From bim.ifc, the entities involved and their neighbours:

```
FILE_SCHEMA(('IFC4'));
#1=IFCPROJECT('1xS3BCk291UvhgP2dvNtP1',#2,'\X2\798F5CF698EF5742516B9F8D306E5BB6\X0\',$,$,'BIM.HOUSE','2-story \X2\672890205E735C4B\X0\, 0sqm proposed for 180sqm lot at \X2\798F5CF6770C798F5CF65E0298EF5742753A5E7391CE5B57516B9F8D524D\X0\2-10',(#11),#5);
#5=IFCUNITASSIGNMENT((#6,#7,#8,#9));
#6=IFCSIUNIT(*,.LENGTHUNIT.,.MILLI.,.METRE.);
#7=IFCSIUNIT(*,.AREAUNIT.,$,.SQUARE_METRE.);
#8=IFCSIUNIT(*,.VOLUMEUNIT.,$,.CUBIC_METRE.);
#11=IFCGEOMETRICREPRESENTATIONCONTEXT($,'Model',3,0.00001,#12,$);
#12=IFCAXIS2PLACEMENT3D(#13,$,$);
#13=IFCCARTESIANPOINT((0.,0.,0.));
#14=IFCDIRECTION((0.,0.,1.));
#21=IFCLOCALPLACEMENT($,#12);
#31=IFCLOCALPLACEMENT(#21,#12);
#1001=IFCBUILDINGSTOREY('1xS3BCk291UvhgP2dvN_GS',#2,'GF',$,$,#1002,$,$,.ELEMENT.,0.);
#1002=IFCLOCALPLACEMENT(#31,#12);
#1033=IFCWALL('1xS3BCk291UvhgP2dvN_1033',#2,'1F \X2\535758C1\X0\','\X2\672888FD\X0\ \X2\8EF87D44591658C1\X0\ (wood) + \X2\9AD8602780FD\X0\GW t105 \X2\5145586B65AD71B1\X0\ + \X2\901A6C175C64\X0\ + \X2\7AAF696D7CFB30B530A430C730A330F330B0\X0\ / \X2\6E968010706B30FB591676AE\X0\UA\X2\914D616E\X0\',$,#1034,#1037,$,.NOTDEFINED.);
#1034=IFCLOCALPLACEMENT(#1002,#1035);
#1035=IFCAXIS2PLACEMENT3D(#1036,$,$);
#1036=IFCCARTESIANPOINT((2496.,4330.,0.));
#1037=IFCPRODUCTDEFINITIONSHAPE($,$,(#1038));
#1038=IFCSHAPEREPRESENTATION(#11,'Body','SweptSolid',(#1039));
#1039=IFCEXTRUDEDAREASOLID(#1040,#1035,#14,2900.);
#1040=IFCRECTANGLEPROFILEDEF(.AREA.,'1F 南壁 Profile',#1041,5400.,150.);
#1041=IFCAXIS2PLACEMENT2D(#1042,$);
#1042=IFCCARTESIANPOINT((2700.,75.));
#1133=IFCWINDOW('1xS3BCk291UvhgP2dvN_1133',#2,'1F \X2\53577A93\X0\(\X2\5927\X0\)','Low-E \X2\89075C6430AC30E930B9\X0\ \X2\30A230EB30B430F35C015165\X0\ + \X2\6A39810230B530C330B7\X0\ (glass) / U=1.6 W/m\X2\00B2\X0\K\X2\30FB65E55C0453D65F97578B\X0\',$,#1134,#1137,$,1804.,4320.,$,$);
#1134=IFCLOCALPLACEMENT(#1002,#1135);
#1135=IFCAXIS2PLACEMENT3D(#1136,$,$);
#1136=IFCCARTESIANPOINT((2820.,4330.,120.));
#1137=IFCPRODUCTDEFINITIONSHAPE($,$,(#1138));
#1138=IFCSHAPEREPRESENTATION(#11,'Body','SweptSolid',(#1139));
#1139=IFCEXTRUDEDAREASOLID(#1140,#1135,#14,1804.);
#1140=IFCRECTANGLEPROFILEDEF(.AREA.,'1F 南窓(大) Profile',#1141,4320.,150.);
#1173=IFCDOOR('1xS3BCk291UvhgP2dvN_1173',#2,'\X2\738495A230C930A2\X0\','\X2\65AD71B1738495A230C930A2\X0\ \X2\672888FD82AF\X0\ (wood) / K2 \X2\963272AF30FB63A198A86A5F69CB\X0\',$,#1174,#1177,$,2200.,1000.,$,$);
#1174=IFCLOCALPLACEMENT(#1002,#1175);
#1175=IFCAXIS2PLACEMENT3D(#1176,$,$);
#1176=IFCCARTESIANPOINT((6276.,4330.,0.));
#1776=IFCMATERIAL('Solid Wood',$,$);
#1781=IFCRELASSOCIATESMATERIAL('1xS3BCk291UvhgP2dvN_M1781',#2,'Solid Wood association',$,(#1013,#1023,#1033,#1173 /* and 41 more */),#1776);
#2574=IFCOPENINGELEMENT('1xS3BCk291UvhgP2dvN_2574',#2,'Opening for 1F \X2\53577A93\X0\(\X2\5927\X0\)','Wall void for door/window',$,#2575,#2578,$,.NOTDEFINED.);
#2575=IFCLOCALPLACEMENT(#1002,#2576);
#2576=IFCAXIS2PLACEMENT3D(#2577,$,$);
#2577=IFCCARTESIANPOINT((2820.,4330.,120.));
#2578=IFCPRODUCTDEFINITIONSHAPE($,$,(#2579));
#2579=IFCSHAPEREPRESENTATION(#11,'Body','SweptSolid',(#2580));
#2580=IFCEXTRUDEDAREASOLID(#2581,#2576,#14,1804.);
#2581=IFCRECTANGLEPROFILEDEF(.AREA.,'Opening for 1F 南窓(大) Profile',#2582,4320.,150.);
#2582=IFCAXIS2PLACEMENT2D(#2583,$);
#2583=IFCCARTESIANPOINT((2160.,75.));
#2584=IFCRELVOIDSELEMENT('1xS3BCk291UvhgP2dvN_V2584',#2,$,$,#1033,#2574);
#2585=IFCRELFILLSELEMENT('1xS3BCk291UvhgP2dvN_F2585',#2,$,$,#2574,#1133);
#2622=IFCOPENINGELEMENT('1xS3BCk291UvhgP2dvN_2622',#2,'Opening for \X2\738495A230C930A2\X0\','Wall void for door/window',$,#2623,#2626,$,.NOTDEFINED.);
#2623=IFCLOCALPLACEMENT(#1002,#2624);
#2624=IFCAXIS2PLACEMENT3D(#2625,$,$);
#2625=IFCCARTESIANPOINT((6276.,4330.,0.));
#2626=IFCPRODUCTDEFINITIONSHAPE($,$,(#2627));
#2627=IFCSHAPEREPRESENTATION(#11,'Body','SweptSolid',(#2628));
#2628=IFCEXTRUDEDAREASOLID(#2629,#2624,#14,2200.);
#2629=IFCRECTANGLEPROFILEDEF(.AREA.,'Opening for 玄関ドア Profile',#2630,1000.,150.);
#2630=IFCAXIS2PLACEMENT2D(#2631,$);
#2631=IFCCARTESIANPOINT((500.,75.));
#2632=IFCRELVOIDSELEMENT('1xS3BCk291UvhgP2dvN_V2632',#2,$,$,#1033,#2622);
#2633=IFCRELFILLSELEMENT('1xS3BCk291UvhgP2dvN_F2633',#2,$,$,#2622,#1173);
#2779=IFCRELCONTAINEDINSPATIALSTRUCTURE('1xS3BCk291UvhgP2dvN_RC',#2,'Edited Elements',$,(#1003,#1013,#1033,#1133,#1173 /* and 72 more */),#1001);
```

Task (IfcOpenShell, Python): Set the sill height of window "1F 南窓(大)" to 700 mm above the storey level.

```python
import numpy as np
import ifcopenshell
import ifcopenshell.api.geometry
import ifcopenshell.geom
import ifcopenshell.util.element
import ifcopenshell.util.placement
import ifcopenshell.util.shape
import ifcopenshell.util.unit

model = ifcopenshell.open("bim.ifc")
unit_scale = ifcopenshell.util.unit.calculate_unit_scale(model)

window = model.by_guid("1xS3BCk291UvhgP2dvN_1133")
opening = window.FillsVoids[0].RelatingOpeningElement
storey = ifcopenshell.util.element.get_container(window, ifc_class="IfcBuildingStorey")
level = ifcopenshell.util.placement.get_local_placement(storey.ObjectPlacement)[2, 3]

# The opening's origin need not be at the sill, so measure its lowest point.
shape = ifcopenshell.geom.create_shape(ifcopenshell.geom.settings(), opening)
bottom = ifcopenshell.util.shape.get_shape_bottom_elevation(shape, shape.geometry) / unit_scale
dz = level + 0.7 / unit_scale - bottom

shift = np.array([0.0, 0.0, dz])
# The window is not placed relative to its opening, so move both.
for product in (opening, window):
    matrix = ifcopenshell.util.placement.get_local_placement(product.ObjectPlacement)
    matrix[:3, 3] += shift
    ifcopenshell.api.geometry.edit_object_placement(model, product=product, matrix=matrix, is_si=False)

print(f"moved by {dz * unit_scale:+.3f} m")

model.write("bim_v2.ifc")
```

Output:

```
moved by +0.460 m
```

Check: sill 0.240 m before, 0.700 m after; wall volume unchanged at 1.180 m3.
